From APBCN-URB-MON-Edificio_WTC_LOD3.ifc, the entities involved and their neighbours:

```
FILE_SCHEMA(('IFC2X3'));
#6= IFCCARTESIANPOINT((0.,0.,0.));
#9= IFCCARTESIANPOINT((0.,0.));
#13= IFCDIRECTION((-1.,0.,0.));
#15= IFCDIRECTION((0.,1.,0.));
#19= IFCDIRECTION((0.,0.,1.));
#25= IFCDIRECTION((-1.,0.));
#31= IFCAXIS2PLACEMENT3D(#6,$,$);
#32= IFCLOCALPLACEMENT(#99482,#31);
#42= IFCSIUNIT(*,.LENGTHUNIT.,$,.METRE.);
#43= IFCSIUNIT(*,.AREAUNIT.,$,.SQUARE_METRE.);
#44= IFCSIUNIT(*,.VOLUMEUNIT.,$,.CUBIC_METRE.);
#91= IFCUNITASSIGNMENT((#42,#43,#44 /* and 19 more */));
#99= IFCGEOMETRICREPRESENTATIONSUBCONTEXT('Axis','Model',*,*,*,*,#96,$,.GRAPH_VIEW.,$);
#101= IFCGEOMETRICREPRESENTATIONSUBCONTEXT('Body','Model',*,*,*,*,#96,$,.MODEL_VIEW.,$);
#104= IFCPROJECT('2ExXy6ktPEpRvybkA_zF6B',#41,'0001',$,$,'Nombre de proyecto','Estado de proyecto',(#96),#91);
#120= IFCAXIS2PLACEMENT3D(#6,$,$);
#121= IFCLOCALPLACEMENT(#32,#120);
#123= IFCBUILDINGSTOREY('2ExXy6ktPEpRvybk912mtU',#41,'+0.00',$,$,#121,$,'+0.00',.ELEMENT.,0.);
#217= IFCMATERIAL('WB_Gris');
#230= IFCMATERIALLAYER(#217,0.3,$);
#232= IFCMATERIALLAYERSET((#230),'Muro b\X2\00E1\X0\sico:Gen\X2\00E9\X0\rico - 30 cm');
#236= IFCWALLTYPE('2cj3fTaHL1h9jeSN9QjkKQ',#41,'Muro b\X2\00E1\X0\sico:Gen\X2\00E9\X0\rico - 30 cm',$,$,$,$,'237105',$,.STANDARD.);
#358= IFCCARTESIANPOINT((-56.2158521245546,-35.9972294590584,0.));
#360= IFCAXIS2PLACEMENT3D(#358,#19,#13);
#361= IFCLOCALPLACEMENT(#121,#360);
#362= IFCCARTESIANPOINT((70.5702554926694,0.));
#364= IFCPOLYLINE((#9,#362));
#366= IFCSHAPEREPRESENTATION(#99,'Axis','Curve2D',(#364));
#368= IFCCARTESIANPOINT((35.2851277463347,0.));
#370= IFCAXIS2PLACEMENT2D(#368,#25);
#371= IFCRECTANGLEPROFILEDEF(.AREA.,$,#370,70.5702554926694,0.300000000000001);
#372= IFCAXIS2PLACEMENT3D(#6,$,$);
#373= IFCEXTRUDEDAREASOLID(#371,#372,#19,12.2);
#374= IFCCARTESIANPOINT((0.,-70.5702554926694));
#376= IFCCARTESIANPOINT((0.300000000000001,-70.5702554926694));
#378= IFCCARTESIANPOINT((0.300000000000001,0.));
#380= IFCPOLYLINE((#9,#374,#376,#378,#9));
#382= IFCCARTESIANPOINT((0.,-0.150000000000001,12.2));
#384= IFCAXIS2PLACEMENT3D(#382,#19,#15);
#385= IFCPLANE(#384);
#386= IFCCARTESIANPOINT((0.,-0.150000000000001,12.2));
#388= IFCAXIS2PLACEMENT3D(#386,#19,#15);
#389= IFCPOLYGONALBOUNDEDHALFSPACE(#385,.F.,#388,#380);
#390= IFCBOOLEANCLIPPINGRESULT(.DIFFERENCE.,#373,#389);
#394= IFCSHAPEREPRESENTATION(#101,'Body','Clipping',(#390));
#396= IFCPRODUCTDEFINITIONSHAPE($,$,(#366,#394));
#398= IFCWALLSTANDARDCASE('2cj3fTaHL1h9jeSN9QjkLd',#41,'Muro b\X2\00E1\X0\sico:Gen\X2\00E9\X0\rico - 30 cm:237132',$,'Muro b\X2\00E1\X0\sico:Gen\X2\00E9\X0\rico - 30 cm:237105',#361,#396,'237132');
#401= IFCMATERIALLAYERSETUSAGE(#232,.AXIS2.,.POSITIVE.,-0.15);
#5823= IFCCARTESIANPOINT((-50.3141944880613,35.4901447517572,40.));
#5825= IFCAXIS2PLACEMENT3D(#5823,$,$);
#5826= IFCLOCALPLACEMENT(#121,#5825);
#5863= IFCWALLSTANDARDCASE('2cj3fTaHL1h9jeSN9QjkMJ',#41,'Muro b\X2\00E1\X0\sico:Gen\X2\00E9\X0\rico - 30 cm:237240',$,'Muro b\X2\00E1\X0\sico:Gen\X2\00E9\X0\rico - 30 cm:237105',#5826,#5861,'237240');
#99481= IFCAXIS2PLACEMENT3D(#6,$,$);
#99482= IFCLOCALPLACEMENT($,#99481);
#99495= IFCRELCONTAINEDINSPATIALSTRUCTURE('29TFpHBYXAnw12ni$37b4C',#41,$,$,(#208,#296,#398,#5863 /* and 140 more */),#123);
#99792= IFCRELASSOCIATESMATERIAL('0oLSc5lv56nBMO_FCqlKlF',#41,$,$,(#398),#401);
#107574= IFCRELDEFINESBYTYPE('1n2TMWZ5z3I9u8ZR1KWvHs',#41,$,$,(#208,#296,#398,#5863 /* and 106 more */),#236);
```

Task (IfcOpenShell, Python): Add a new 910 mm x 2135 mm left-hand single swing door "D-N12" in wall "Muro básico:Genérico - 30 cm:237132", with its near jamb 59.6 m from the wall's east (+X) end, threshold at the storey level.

```python
import numpy as np
import ifcopenshell
import ifcopenshell.api.feature
import ifcopenshell.api.geometry
import ifcopenshell.api.root
import ifcopenshell.api.spatial
import ifcopenshell.api.type
import ifcopenshell.geom
import ifcopenshell.util.element
import ifcopenshell.util.placement
import ifcopenshell.util.representation
import ifcopenshell.util.shape
import ifcopenshell.util.unit

model = ifcopenshell.open("APBCN-URB-MON-Edificio_WTC_LOD3.ifc")
unit_scale = ifcopenshell.util.unit.calculate_unit_scale(model)
settings = ifcopenshell.geom.settings()


def volume(element):
    """Net volume in cubic metres, openings subtracted."""
    shape = ifcopenshell.geom.create_shape(settings, element)
    return ifcopenshell.util.shape.get_volume(shape.geometry)


wall = model.by_guid("2cj3fTaHL1h9jeSN9QjkLd")
storey = ifcopenshell.util.element.get_container(wall, ifc_class="IfcBuildingStorey")
context = ifcopenshell.util.representation.get_context(model, "Model", "Body", "MODEL_VIEW")
before = volume(wall)

width, height, from_end, sill = 0.91, 2.135, 59.6, 0.0  # metres

# The wall runs along its own X axis, and the end named is its -X end.
wall_shape = ifcopenshell.geom.create_shape(settings, wall)
x, y, z = ifcopenshell.util.shape.get_vertices(wall_shape.geometry).T
start = x.min() + from_end
face, thickness = float(y.min()), float(y.max() - y.min())
wall_matrix = ifcopenshell.util.placement.get_local_placement(wall.ObjectPlacement)
level = ifcopenshell.util.placement.get_local_placement(storey.ObjectPlacement)[2, 3]


def in_wall(x, y):
    """Placement at x, y metres in the wall's axes, at sill height."""
    matrix = wall_matrix.copy()
    matrix[:, 3] = wall_matrix @ np.array([x / unit_scale, y / unit_scale, 0.0, 1.0])
    matrix[2, 3] = level + sill / unit_scale
    return matrix


# Opening: a box that overshoots both wall faces by 50 mm.
opening = ifcopenshell.api.root.create_entity(model, ifc_class="IfcOpeningElement")
box = ifcopenshell.api.geometry.add_wall_representation(
    model, context=context, length=width, height=height, thickness=thickness + 0.1
)
ifcopenshell.api.geometry.assign_representation(model, product=opening, representation=box)
ifcopenshell.api.geometry.edit_object_placement(model, product=opening, matrix=in_wall(start, face - 0.05), is_si=False)
ifcopenshell.api.feature.add_feature(model, feature=opening, element=wall)

door = ifcopenshell.api.root.create_entity(model, ifc_class="IfcDoor", name="D-N12")
door.OverallWidth, door.OverallHeight = width / unit_scale, height / unit_scale
body = ifcopenshell.api.geometry.add_door_representation(
    model,
    context=context,
    overall_width=door.OverallWidth,
    overall_height=door.OverallHeight,
    operation_type="SINGLE_SWING_LEFT",
    lining_properties={"LiningDepth": thickness / unit_scale, "ThresholdDepth": thickness / unit_scale},
)
ifcopenshell.api.geometry.assign_representation(model, product=door, representation=body)
ifcopenshell.api.spatial.assign_container(model, products=[door], relating_structure=storey)
fills = ifcopenshell.api.feature.add_filling(model, opening=opening, element=door)
fills.OwnerHistory = door.OwnerHistory  # required in IFC2X3

# IFC2X3 keeps the operation on the door style.
style = ifcopenshell.api.root.create_entity(model, ifc_class="IfcDoorStyle", name="D-N12")
style.OperationType, style.ConstructionType = "SINGLE_SWING_LEFT", "NOTDEFINED"
style.ParameterTakesPrecedence = style.Sizeable = False
ifcopenshell.api.type.assign_type(model, related_objects=[door], relating_type=style)

# The lining spans the wall, so the door starts at the wall face.
ifcopenshell.api.geometry.edit_object_placement(model, product=door, matrix=in_wall(start, face), is_si=False)

after = volume(wall)

print(f"wall volume {before:.3f} -> {after:.3f} m3")

model.write("APBCN-URB-MON-Edificio_WTC_LOD3_rev.ifc")
```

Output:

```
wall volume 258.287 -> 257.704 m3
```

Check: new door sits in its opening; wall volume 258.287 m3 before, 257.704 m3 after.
